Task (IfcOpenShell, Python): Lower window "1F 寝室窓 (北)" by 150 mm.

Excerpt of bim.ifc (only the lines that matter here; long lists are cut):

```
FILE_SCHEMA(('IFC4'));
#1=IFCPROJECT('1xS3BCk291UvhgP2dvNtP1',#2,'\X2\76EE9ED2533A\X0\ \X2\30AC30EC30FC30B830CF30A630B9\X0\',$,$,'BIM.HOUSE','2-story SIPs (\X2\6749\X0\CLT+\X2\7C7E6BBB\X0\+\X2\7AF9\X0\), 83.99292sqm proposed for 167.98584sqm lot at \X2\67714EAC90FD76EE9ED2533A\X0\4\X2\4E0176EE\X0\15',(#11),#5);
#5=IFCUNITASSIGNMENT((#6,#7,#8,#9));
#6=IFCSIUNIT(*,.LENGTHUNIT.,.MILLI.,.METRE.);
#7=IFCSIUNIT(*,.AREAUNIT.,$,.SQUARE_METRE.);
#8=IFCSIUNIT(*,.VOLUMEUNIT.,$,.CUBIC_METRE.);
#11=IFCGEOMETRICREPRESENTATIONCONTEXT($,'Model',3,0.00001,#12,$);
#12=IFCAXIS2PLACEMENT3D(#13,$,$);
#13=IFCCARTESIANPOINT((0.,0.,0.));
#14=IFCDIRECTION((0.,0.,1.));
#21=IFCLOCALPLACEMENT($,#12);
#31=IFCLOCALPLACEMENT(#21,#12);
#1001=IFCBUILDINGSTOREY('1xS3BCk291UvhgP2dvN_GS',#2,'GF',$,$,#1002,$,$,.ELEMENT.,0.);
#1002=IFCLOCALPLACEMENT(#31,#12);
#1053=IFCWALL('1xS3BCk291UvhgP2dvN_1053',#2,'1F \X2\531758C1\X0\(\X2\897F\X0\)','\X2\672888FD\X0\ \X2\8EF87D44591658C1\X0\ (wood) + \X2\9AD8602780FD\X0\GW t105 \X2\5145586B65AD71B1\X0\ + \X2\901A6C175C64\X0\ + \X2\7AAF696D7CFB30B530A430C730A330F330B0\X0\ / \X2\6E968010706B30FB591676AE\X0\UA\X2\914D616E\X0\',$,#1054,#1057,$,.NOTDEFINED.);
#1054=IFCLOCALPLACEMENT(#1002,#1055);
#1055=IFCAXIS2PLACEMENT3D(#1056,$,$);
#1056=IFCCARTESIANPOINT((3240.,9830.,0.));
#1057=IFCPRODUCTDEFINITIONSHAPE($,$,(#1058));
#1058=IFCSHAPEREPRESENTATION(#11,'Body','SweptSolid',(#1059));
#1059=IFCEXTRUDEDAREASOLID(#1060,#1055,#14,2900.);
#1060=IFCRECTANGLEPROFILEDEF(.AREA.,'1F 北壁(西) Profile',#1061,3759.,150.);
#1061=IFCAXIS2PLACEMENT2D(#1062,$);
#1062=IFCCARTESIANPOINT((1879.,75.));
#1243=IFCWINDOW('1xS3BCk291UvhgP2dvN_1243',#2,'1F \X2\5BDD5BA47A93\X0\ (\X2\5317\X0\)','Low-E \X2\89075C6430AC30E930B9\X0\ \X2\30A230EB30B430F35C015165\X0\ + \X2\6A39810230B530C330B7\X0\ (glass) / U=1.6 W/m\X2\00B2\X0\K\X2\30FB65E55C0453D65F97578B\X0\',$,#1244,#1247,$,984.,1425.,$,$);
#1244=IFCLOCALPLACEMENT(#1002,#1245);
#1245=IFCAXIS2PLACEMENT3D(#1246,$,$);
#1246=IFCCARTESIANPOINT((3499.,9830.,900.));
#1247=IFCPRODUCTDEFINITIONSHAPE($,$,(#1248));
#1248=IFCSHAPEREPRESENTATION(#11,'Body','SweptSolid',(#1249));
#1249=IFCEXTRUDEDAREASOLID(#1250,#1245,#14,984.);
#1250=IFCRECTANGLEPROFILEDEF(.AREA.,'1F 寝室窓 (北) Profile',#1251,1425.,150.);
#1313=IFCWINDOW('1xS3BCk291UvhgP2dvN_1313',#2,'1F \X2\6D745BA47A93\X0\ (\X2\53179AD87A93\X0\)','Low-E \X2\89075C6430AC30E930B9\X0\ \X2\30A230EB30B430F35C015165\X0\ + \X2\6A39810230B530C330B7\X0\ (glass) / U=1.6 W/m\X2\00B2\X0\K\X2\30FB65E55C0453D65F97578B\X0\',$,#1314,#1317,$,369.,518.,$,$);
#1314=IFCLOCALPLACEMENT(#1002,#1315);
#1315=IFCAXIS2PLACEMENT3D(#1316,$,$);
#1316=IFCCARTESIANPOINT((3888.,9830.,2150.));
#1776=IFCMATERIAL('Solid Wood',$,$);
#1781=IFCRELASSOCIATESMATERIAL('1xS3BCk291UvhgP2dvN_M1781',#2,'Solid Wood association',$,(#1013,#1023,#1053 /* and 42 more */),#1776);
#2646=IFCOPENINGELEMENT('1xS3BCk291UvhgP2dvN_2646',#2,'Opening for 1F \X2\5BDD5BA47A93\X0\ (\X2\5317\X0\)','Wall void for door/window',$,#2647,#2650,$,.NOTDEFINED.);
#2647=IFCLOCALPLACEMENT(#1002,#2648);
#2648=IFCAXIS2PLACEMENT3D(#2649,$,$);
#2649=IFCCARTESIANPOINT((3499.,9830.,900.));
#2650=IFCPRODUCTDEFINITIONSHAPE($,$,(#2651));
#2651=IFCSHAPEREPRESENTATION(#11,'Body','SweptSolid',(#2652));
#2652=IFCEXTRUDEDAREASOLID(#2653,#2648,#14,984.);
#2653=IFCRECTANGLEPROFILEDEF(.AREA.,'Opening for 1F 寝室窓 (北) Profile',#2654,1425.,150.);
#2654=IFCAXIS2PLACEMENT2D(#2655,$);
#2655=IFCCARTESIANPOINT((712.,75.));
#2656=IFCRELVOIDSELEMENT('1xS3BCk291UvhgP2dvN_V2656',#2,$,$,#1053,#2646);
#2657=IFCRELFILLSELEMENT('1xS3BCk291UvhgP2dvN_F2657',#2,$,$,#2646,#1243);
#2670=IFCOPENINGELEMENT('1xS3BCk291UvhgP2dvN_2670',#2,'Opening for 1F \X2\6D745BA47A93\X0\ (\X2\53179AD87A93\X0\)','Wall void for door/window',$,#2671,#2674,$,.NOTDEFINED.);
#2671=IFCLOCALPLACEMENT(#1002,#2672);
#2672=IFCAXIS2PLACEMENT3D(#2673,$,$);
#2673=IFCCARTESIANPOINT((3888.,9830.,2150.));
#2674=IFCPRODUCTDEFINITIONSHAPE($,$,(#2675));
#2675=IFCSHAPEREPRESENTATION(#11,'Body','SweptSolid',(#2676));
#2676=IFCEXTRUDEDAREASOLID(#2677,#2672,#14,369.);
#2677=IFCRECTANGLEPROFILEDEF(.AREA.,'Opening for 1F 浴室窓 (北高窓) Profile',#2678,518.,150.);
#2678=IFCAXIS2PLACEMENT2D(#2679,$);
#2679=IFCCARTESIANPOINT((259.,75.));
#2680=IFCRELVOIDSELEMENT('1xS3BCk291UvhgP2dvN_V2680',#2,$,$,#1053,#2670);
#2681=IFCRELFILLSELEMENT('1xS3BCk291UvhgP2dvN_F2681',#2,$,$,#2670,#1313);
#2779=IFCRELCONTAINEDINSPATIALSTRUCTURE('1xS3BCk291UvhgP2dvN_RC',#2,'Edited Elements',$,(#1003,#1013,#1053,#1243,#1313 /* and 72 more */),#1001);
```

```python
import numpy as np
import ifcopenshell
import ifcopenshell.api.geometry
import ifcopenshell.util.placement
import ifcopenshell.util.unit

model = ifcopenshell.open("bim.ifc")
unit_scale = ifcopenshell.util.unit.calculate_unit_scale(model)

window = model.by_guid("1xS3BCk291UvhgP2dvN_1243")
opening = window.FillsVoids[0].RelatingOpeningElement
dz = -0.15 / unit_scale

shift = np.array([0.0, 0.0, dz])
# The window is not placed relative to its opening, so move both.
for product in (opening, window):
    matrix = ifcopenshell.util.placement.get_local_placement(product.ObjectPlacement)
    matrix[:3, 3] += shift
    ifcopenshell.api.geometry.edit_object_placement(model, product=product, matrix=matrix, is_si=False)

print(f"moved by {dz * unit_scale:+.3f} m")

model.write("bim-out.ifc")
```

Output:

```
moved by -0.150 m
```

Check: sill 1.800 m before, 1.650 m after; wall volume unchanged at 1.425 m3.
